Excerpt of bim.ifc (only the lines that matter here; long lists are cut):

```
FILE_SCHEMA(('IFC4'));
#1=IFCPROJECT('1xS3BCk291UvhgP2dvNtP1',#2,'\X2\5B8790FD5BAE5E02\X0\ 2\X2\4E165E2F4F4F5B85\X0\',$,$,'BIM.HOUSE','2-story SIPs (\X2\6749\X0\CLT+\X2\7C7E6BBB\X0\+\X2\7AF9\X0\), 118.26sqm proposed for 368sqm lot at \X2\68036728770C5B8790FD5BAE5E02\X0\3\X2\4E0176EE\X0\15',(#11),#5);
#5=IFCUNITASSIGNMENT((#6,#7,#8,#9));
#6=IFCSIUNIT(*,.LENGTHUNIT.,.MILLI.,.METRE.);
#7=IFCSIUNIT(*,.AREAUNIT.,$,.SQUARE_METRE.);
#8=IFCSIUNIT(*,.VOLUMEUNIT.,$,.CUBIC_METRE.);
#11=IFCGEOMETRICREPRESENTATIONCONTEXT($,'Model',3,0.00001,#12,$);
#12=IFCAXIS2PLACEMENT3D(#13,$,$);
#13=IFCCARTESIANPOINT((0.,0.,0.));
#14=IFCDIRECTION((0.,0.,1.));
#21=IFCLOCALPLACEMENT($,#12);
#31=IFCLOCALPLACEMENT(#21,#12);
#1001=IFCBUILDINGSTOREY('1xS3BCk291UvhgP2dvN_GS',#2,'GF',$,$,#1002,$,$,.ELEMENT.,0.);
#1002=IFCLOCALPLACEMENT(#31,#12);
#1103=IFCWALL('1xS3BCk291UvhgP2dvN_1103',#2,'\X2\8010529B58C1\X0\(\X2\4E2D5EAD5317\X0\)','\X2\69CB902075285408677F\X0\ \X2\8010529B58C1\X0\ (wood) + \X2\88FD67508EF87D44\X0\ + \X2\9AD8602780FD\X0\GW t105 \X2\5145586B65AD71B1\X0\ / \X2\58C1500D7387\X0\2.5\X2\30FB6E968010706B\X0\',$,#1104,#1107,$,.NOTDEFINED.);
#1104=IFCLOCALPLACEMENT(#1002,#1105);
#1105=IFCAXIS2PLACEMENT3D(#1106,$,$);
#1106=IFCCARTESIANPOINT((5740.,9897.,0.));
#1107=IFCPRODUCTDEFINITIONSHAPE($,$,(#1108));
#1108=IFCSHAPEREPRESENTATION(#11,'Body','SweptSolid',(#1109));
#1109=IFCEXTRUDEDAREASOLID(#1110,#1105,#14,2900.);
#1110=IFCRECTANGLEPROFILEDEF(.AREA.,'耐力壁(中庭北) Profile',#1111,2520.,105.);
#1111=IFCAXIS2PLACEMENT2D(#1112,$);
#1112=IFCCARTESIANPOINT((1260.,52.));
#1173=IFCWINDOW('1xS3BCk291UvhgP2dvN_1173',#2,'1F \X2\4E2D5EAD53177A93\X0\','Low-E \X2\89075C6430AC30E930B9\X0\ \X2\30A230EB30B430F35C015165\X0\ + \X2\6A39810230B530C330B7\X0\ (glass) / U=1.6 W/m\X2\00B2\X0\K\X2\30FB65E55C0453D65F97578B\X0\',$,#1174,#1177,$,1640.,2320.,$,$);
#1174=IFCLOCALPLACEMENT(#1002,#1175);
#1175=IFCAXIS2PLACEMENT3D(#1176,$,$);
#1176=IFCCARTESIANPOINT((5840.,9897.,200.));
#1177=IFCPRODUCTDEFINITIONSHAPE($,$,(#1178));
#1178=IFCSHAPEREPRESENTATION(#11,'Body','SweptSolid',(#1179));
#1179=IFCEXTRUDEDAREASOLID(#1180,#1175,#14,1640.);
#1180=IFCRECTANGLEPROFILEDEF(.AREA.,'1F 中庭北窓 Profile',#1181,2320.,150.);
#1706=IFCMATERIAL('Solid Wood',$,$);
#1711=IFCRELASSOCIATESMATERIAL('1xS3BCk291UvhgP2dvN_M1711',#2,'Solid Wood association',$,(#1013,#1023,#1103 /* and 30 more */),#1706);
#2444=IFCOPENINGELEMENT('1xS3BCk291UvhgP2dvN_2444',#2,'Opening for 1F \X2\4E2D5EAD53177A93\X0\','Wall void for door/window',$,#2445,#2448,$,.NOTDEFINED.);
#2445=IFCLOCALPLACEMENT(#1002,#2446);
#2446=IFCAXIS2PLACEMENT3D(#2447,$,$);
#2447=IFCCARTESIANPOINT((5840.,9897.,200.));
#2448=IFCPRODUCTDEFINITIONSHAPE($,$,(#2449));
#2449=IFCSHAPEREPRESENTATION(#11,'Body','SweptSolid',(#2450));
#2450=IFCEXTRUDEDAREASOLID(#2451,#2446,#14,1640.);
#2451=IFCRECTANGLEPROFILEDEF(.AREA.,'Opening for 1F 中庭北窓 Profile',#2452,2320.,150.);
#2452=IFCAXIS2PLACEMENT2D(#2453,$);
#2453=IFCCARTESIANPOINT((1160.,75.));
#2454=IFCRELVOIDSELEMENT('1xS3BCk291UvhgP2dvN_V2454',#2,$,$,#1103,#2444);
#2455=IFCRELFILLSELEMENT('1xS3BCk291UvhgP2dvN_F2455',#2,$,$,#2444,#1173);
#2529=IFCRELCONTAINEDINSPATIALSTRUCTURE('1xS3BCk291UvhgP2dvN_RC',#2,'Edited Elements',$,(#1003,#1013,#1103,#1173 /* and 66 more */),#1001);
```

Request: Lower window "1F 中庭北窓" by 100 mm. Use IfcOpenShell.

```python
import numpy as np
import ifcopenshell
import ifcopenshell.api.geometry
import ifcopenshell.util.placement
import ifcopenshell.util.unit

model = ifcopenshell.open("bim.ifc")
unit_scale = ifcopenshell.util.unit.calculate_unit_scale(model)

window = model.by_id(1173)
opening = window.FillsVoids[0].RelatingOpeningElement
dz = -0.1 / unit_scale

shift = np.array([0.0, 0.0, dz])
# The window is not placed relative to its opening, so move both.
for product in (opening, window):
    matrix = ifcopenshell.util.placement.get_local_placement(product.ObjectPlacement)
    matrix[:3, 3] += shift
    ifcopenshell.api.geometry.edit_object_placement(model, product=product, matrix=matrix, is_si=False)

print(f"moved by {dz * unit_scale:+.3f} m")

model.write("bim_edited.ifc")
```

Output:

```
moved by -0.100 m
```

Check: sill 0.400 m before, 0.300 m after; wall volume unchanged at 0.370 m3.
